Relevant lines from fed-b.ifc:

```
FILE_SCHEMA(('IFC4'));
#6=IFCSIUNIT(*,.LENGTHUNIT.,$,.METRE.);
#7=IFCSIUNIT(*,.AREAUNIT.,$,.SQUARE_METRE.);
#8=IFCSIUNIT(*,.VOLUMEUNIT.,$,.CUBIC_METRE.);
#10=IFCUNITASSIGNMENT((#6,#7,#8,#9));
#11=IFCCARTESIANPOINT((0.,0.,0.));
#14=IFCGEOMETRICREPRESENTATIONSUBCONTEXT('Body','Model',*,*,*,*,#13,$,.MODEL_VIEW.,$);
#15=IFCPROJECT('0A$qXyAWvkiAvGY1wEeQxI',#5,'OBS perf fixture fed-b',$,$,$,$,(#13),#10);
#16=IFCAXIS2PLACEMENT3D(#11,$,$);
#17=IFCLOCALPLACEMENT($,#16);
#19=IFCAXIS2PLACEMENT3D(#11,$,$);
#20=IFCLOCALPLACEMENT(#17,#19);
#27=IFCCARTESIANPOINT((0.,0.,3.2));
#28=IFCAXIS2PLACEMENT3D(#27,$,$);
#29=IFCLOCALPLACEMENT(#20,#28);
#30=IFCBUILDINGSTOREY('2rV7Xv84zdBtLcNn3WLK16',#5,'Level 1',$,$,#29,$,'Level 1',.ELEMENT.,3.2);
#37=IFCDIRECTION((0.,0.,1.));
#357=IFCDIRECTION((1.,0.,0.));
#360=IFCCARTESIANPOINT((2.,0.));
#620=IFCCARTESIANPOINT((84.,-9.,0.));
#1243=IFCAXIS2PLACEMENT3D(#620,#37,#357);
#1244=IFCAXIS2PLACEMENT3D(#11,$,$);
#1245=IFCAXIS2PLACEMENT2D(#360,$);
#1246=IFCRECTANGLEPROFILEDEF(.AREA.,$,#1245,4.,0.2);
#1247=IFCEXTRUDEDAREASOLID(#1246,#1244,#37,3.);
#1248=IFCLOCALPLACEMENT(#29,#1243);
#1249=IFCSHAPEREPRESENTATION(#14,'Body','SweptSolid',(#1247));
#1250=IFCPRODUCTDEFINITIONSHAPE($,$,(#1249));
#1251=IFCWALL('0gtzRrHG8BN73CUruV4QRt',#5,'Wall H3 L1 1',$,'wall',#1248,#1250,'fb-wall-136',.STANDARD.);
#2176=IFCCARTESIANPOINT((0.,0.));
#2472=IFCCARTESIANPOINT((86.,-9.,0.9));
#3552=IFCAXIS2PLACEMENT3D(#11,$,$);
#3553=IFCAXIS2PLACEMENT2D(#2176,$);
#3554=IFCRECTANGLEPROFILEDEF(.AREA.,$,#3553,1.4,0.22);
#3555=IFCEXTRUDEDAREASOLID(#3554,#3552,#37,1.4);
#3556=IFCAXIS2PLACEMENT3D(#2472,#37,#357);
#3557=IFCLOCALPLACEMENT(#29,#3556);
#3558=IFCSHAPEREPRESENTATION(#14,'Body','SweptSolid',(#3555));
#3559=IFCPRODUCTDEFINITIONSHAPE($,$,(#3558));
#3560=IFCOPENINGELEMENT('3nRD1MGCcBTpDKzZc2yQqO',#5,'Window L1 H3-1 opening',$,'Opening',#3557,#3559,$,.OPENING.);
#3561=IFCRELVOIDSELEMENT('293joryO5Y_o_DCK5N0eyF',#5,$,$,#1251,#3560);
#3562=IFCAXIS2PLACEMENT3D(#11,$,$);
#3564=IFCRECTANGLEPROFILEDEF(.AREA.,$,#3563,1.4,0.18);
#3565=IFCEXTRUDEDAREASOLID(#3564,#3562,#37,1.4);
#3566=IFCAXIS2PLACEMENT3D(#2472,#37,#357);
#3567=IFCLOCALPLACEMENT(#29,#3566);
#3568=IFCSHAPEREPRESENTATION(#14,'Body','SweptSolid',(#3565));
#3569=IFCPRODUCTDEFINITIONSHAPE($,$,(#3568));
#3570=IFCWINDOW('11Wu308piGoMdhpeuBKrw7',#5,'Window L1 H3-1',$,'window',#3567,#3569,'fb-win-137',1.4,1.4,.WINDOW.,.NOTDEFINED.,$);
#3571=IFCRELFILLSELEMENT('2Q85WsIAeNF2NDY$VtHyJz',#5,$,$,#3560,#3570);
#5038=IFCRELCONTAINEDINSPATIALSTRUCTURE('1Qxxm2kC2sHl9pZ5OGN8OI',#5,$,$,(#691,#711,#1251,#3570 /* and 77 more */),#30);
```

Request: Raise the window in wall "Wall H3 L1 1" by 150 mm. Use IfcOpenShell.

```python
import numpy as np
import ifcopenshell
import ifcopenshell.api.geometry
import ifcopenshell.util.placement
import ifcopenshell.util.unit

model = ifcopenshell.open("fed-b.ifc")
unit_scale = ifcopenshell.util.unit.calculate_unit_scale(model)

window = model.by_guid("11Wu308piGoMdhpeuBKrw7")
opening = window.FillsVoids[0].RelatingOpeningElement
dz = 0.15

shift = np.array([0.0, 0.0, dz])
# The window is not placed relative to its opening, so move both.
for product in (opening, window):
    matrix = ifcopenshell.util.placement.get_local_placement(product.ObjectPlacement)
    matrix[:3, 3] += shift
    ifcopenshell.api.geometry.edit_object_placement(model, product=product, matrix=matrix, is_si=False)

print(f"moved by {dz * unit_scale:+.3f} m")

model.write("fed-b_v2.ifc")
```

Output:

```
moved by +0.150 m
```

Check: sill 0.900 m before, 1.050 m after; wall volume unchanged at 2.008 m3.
